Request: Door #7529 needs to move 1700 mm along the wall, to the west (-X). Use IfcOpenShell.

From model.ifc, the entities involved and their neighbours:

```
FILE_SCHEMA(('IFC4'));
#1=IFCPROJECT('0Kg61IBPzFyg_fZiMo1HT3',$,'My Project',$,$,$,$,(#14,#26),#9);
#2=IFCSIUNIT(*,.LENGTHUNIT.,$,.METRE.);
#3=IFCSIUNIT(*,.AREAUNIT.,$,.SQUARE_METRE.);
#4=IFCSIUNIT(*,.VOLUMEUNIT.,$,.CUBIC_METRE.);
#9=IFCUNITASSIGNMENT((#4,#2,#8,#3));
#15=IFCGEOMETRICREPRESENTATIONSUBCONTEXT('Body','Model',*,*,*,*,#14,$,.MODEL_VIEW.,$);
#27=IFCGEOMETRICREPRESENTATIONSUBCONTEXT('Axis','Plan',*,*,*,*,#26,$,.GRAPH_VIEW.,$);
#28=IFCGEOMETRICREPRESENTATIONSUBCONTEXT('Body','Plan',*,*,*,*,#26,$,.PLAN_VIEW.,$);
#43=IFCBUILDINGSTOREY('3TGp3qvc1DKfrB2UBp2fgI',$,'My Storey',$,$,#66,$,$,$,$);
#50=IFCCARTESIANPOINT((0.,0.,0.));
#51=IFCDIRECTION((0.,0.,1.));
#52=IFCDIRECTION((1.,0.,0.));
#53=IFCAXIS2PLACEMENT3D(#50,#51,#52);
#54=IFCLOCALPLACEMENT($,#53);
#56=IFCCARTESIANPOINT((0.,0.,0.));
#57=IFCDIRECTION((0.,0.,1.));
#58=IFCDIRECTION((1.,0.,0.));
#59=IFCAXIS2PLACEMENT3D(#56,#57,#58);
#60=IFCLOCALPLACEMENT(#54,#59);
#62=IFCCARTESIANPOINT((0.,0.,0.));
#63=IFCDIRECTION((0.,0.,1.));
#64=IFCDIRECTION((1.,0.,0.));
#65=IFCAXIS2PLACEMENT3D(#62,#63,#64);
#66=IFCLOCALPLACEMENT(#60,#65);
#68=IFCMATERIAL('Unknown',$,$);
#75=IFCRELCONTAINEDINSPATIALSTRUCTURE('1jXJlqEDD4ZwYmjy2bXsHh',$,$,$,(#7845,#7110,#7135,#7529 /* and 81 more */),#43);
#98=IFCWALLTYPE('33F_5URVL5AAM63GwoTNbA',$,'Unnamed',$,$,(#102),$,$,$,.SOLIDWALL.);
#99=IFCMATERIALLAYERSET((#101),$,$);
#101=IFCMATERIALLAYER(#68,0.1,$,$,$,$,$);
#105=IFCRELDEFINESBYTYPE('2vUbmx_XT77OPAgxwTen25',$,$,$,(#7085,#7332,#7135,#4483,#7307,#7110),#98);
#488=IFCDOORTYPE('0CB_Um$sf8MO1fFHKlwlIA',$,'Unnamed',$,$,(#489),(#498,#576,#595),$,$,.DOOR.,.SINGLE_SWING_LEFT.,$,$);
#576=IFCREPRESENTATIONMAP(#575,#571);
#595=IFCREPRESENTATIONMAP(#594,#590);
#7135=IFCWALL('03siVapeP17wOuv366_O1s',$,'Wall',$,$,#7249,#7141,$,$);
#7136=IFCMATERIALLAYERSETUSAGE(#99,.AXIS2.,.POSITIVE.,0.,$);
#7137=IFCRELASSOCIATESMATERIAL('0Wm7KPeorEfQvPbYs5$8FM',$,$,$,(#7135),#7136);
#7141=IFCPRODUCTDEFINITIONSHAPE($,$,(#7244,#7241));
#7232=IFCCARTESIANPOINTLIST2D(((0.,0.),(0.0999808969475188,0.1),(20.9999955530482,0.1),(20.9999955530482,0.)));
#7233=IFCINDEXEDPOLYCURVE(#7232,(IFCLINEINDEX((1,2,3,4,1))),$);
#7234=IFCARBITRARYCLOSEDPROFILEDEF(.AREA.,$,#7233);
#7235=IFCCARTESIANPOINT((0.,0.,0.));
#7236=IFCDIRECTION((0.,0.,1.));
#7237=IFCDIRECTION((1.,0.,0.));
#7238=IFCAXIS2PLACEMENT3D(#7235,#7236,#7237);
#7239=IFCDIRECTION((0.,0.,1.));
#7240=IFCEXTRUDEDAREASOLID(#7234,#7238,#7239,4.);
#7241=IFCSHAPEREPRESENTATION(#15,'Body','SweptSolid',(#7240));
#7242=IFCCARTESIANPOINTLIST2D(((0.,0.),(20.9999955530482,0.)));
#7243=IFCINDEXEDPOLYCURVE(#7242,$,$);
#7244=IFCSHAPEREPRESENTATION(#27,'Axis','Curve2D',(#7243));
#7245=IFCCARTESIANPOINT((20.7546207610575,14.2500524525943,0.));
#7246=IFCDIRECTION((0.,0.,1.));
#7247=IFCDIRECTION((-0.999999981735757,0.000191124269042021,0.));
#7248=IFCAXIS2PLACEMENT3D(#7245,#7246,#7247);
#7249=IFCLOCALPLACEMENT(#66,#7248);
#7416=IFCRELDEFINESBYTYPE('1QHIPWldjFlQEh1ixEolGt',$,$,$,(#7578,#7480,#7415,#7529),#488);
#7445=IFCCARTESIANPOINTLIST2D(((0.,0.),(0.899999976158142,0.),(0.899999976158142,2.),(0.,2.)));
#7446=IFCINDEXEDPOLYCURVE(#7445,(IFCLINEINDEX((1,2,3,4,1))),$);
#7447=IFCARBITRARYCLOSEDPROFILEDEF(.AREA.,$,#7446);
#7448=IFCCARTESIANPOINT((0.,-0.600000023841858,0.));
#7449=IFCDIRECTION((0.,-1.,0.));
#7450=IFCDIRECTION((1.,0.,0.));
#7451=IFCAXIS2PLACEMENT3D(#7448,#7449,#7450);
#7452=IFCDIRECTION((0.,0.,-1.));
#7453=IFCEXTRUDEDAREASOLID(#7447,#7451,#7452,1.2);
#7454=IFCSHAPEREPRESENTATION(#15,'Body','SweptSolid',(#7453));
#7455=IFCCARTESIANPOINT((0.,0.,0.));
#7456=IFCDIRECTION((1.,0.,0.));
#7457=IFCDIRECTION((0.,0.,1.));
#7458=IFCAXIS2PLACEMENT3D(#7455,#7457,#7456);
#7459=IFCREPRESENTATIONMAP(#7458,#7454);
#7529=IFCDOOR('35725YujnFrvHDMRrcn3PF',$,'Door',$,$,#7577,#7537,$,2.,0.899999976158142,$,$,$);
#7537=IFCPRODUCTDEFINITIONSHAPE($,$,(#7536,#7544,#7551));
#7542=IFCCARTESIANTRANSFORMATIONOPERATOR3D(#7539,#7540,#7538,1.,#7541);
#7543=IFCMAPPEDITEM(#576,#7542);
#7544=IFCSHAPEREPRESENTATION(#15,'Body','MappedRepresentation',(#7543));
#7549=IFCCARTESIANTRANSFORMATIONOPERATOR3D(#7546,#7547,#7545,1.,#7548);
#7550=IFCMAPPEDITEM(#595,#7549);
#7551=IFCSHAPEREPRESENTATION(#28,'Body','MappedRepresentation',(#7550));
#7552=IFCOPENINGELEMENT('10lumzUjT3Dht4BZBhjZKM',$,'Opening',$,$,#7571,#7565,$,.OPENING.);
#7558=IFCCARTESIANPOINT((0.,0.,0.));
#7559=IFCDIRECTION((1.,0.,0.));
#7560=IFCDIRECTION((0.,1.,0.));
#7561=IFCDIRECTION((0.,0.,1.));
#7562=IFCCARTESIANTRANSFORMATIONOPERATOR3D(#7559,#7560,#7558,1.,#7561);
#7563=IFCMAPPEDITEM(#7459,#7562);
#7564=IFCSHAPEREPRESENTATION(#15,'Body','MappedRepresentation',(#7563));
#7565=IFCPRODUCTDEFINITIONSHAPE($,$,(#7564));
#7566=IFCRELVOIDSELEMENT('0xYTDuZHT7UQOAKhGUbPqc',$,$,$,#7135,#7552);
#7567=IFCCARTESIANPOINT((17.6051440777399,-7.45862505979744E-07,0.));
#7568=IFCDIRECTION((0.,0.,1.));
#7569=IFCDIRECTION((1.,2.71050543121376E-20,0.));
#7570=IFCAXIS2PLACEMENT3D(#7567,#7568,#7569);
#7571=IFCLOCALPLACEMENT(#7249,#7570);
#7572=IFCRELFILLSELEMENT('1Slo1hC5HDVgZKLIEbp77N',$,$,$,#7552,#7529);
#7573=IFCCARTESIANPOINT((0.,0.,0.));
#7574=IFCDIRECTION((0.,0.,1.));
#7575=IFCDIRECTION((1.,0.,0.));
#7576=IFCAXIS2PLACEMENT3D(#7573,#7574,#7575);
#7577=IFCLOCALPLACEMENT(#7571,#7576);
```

```python
import ifcopenshell
import ifcopenshell.api.geometry
import ifcopenshell.util.placement
import ifcopenshell.util.unit

model = ifcopenshell.open("model.ifc")
unit_scale = ifcopenshell.util.unit.calculate_unit_scale(model)

door = model.by_guid("35725YujnFrvHDMRrcn3PF")
opening = door.FillsVoids[0].RelatingOpeningElement
wall = opening.VoidsElements[0].RelatingBuildingElement

wall_matrix = ifcopenshell.util.placement.get_local_placement(wall.ObjectPlacement)
shift = wall_matrix[:3, 0] * 1.7 / unit_scale
before = ifcopenshell.util.placement.get_local_placement(door.ObjectPlacement)[:3, 3].copy()

# The door is placed relative to its opening, so it follows when the opening moves.
matrix = ifcopenshell.util.placement.get_local_placement(opening.ObjectPlacement)
matrix[:3, 3] += shift
ifcopenshell.api.geometry.edit_object_placement(
    model, product=opening, matrix=matrix, is_si=False, should_transform_children=True
)

after = ifcopenshell.util.placement.get_local_placement(door.ObjectPlacement)[:3, 3]
print("door moved by", (after - before).round(3) + 0.0)

model.write("model_v2.ifc")
```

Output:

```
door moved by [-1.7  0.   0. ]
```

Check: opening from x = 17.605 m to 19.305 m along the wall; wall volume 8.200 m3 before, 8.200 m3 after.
